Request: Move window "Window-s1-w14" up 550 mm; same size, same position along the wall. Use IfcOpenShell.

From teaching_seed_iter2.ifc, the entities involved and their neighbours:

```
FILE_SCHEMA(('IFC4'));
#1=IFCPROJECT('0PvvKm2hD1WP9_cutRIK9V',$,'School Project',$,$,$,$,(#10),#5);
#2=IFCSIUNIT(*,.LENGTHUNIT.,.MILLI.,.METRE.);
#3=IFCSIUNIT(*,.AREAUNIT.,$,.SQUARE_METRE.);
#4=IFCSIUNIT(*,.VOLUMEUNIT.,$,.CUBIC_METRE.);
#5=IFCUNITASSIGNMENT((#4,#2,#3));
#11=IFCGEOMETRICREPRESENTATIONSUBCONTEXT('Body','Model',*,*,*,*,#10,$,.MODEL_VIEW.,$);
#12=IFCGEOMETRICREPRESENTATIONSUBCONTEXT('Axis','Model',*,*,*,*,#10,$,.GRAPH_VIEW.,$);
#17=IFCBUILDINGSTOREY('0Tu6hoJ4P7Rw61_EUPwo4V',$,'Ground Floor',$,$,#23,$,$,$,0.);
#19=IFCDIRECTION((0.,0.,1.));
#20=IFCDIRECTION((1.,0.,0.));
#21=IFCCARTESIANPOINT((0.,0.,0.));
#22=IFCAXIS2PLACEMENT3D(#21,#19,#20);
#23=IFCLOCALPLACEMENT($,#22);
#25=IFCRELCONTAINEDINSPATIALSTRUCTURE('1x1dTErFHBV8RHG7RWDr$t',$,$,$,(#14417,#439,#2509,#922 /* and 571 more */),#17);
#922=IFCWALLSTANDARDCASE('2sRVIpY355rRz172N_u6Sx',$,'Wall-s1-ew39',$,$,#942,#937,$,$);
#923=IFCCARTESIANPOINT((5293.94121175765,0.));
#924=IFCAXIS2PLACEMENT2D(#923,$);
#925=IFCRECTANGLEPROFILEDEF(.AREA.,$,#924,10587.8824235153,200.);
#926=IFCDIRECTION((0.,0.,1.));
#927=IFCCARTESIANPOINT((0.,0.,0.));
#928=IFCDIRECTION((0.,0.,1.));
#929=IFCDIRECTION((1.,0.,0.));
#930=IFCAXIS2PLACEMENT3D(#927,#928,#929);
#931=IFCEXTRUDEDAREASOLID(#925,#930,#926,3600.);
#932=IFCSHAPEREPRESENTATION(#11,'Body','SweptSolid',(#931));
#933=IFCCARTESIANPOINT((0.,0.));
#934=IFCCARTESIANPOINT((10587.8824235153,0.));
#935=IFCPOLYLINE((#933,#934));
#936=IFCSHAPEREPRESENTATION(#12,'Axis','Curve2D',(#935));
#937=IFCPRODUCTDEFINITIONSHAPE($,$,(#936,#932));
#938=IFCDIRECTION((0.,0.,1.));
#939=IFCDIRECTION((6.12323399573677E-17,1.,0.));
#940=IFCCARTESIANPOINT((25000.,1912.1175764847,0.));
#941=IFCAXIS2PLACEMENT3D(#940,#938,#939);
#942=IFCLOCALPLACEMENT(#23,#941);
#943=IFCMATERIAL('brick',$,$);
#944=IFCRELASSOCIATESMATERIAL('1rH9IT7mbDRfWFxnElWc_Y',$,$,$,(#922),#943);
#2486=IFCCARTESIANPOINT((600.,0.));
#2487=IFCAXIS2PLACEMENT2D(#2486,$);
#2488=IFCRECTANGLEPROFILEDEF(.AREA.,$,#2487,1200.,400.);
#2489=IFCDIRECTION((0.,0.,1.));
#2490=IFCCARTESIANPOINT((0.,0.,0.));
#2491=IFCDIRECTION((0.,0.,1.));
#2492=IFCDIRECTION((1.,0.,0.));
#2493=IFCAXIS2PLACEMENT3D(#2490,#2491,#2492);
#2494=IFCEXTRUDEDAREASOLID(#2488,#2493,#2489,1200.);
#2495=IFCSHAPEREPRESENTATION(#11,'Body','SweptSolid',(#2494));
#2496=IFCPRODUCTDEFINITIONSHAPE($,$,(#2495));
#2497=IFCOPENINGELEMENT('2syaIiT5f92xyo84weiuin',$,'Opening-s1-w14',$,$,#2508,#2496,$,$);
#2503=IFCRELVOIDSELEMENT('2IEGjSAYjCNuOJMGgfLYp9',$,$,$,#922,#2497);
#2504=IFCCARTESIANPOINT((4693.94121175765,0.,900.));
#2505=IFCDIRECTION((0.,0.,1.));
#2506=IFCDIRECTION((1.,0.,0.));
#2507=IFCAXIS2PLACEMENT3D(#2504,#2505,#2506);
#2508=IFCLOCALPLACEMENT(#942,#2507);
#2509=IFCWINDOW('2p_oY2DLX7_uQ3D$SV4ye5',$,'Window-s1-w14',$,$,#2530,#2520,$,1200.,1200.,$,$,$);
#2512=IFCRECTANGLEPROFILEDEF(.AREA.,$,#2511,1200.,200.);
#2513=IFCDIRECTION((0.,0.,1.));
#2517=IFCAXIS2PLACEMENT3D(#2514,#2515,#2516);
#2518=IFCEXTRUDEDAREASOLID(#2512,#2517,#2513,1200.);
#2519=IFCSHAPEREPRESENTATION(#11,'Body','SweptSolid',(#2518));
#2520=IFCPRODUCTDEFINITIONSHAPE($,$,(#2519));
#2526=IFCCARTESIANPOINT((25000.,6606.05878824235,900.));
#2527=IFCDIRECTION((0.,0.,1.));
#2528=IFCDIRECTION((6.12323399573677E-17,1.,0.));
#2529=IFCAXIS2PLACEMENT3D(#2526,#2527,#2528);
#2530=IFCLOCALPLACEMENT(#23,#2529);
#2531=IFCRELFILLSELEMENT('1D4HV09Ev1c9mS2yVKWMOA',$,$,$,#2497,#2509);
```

```python
import numpy as np
import ifcopenshell
import ifcopenshell.api.geometry
import ifcopenshell.util.placement
import ifcopenshell.util.unit

model = ifcopenshell.open("teaching_seed_iter2.ifc")
unit_scale = ifcopenshell.util.unit.calculate_unit_scale(model)

window = model.by_guid("2p_oY2DLX7_uQ3D$SV4ye5")
opening = window.FillsVoids[0].RelatingOpeningElement
dz = 0.55 / unit_scale

shift = np.array([0.0, 0.0, dz])
# The window is not placed relative to its opening, so move both.
for product in (opening, window):
    matrix = ifcopenshell.util.placement.get_local_placement(product.ObjectPlacement)
    matrix[:3, 3] += shift
    ifcopenshell.api.geometry.edit_object_placement(model, product=product, matrix=matrix, is_si=False)

print(f"moved by {dz * unit_scale:+.3f} m")

model.write("teaching_seed_iter2_updated.ifc")
```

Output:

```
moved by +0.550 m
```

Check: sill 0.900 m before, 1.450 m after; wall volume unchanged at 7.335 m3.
